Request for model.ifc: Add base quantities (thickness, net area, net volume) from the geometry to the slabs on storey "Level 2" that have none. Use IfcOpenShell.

First a look at what the model holds.

```python
import ifcopenshell
import ifcopenshell.util.element
import ifcopenshell.util.unit

model = ifcopenshell.open("model.ifc")
print(model.schema)
for unit_type in ("LENGTHUNIT", "AREAUNIT", "VOLUMEUNIT"):
    print(unit_type, ifcopenshell.util.unit.calculate_unit_scale(model, unit_type))
storey = next(s for s in model.by_type("IfcBuildingStorey") if s.Name == "Level 2")
slabs = [e for e in ifcopenshell.util.element.get_decomposition(storey) if e.is_a("IfcSlab")]
for e in sorted(slabs, key=lambda e: e.id()):
    print(e.id(), e.is_a(), e.Name, list(ifcopenshell.util.element.get_psets(e, qtos_only=True)), sep=" | ")
```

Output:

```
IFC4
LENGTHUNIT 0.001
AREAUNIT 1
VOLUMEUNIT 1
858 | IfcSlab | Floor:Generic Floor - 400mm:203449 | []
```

```python
import ifcopenshell
import ifcopenshell.api.pset
import ifcopenshell.geom
import ifcopenshell.util.element
import ifcopenshell.util.shape
import ifcopenshell.util.unit

model = ifcopenshell.open("model.ifc")
unit_scale = ifcopenshell.util.unit.calculate_unit_scale(model)
area_scale = ifcopenshell.util.unit.calculate_unit_scale(model, "AREAUNIT")
volume_scale = ifcopenshell.util.unit.calculate_unit_scale(model, "VOLUMEUNIT")
settings = ifcopenshell.geom.settings()

storey = next(s for s in model.by_type("IfcBuildingStorey") if s.Name == "Level 2")
slabs = [e for e in ifcopenshell.util.element.get_decomposition(storey) if e.is_a("IfcSlab")]

for e in sorted(slabs, key=lambda e: e.id()):
    if ifcopenshell.util.element.get_psets(e, qtos_only=True, should_inherit=False):
        continue
    # Geometry comes back in metres, in the element's own axes.
    shape = ifcopenshell.geom.create_shape(settings, e)
    values = {
        "Width": ifcopenshell.util.shape.get_z(shape.geometry) / unit_scale,
        "NetArea": ifcopenshell.util.shape.get_footprint_area(shape.geometry) / area_scale,
        "NetVolume": ifcopenshell.util.shape.get_volume(shape.geometry) / volume_scale,
    }
    qto = ifcopenshell.api.pset.add_qto(model, product=e, name="Qto_SlabBaseQuantities")
    ifcopenshell.api.pset.edit_qto(model, qto=qto, properties=values)
    print(e.id(), {k: round(v, 3) for k, v in values.items()})

model.write("model-out.ifc")
```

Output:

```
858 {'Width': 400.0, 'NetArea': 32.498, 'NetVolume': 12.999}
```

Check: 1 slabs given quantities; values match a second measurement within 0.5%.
